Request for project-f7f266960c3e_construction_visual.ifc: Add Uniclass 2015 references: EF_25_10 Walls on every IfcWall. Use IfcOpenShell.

First a look at what the model holds.

```python
import ifcopenshell

model = ifcopenshell.open("project-f7f266960c3e_construction_visual.ifc")
print(model.schema)
print("classifications:", [c.Name for c in model.by_type("IfcClassification")])
for ifc_class in ("IfcDoor", "IfcRoof", "IfcStair", "IfcWall", "IfcWindow"):
    print(ifc_class, len(model.by_type(ifc_class)))
```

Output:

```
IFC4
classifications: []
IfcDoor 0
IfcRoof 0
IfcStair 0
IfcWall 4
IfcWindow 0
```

```python
import ifcopenshell
import ifcopenshell.api.classification

model = ifcopenshell.open("project-f7f266960c3e_construction_visual.ifc")

system = ifcopenshell.api.classification.add_classification(model, classification="Uniclass 2015")

codes = {
    "IfcWall": ("EF_25_10", "Walls"),
}
for ifc_class, (code, name) in codes.items():
    products = model.by_type(ifc_class)
    ifcopenshell.api.classification.add_reference(
        model, products=products, classification=system, identification=code, name=name
    )
    print(code, len(products))

model.write("project-f7f266960c3e_construction_visual_edited.ifc")
```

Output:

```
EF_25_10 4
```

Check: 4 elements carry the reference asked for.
